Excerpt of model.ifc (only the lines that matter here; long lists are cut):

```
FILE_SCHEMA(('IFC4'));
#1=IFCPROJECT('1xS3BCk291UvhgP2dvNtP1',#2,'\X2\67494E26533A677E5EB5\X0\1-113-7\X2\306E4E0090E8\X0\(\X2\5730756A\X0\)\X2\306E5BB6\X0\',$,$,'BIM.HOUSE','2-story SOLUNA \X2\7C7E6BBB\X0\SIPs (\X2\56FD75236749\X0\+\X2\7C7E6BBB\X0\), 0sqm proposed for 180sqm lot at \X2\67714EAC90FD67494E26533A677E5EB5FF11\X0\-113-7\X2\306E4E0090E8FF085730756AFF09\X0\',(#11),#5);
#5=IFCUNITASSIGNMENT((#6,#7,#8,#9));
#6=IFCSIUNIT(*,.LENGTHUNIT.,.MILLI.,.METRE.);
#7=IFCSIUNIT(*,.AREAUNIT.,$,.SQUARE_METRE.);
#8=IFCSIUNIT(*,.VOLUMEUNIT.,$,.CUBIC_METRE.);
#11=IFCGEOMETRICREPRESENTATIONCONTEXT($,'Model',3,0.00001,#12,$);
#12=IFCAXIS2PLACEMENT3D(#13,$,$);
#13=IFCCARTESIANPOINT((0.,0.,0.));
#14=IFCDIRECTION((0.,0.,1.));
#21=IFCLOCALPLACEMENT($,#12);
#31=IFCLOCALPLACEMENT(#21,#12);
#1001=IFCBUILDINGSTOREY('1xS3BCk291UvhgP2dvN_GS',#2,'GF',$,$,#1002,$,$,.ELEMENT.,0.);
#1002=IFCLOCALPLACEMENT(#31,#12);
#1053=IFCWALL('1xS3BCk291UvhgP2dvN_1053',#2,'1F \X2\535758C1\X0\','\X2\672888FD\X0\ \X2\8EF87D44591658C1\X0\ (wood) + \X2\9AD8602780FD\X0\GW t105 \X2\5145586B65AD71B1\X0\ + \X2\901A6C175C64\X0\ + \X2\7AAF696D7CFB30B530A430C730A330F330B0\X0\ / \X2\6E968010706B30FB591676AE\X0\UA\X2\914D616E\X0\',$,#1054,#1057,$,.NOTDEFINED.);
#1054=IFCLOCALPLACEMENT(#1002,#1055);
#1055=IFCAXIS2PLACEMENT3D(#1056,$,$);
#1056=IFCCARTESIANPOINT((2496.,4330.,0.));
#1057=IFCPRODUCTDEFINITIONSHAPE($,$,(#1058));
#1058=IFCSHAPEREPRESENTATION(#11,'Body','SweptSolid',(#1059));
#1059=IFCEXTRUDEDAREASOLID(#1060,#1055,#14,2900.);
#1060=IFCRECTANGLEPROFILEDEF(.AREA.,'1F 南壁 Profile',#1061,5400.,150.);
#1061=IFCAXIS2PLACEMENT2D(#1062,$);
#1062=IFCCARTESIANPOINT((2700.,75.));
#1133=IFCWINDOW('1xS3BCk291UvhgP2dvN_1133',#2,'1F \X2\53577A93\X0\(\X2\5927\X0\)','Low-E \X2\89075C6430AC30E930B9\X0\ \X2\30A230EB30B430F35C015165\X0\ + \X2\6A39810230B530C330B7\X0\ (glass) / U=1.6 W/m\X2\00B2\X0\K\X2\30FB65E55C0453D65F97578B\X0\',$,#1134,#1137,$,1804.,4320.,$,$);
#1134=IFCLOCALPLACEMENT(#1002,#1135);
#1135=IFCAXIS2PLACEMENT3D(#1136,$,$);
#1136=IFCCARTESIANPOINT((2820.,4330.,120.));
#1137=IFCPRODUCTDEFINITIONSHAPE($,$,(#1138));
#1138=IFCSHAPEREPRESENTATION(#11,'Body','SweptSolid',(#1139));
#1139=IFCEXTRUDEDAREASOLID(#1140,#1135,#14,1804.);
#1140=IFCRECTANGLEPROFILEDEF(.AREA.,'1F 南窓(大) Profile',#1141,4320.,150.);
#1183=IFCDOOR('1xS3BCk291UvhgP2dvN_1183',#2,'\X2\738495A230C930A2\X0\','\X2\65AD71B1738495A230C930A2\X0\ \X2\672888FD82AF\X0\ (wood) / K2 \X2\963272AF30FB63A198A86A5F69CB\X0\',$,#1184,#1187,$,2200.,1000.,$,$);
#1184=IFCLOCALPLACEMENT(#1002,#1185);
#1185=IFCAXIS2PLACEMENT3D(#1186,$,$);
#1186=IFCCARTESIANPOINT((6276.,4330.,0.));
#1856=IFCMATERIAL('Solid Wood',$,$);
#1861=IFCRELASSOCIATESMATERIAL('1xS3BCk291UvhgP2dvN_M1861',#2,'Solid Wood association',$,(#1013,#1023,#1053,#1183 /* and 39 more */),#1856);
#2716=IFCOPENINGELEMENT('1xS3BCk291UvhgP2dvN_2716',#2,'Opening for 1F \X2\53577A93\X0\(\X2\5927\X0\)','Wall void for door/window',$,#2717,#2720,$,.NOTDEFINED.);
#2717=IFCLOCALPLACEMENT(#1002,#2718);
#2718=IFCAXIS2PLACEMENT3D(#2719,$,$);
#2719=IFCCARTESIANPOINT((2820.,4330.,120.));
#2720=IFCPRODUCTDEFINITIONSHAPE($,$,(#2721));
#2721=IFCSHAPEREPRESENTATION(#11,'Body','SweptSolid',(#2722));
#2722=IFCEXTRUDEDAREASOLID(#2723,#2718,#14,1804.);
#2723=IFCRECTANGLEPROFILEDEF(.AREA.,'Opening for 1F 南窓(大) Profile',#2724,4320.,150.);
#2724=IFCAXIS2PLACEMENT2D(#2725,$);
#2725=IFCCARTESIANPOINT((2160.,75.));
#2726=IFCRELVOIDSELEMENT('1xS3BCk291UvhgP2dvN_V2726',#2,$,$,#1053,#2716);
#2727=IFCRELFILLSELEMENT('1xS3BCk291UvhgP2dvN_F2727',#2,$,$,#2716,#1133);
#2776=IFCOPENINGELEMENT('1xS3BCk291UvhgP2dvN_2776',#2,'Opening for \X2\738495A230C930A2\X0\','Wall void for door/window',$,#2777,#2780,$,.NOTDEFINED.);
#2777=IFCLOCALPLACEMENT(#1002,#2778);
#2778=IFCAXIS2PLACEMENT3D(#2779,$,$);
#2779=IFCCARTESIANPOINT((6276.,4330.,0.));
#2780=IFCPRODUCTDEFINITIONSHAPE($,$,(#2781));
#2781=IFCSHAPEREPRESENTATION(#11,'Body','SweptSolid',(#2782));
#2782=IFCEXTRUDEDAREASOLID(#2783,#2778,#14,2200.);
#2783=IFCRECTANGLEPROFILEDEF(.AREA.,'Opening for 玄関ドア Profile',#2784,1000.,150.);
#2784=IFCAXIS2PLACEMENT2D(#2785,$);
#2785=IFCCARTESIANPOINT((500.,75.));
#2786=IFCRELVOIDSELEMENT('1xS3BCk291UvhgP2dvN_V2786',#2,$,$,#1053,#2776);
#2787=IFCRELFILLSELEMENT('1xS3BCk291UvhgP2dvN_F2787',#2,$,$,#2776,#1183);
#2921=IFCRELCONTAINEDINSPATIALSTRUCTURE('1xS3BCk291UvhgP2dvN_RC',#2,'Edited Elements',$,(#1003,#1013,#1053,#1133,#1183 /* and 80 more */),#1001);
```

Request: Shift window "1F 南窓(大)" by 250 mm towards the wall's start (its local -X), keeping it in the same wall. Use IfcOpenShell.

```python
import ifcopenshell
import ifcopenshell.api.geometry
import ifcopenshell.util.placement

model = ifcopenshell.open("model.ifc")

window = model.by_guid("1xS3BCk291UvhgP2dvN_1133")
opening = window.FillsVoids[0].RelatingOpeningElement
wall = opening.VoidsElements[0].RelatingBuildingElement

wall_matrix = ifcopenshell.util.placement.get_local_placement(wall.ObjectPlacement)
shift = wall_matrix[:3, 0] * -250.0
before = ifcopenshell.util.placement.get_local_placement(window.ObjectPlacement)[:3, 3].copy()

# The window is not placed relative to its opening, so move both.
for product in (opening, window):
    matrix = ifcopenshell.util.placement.get_local_placement(product.ObjectPlacement)
    matrix[:3, 3] += shift
    ifcopenshell.api.geometry.edit_object_placement(model, product=product, matrix=matrix, is_si=False)

after = ifcopenshell.util.placement.get_local_placement(window.ObjectPlacement)[:3, 3]
print("window moved by", (after - before).round(3) + 0.0)

model.write("model_v2.ifc")
```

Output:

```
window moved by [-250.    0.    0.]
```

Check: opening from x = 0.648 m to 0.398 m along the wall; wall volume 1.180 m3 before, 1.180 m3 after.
